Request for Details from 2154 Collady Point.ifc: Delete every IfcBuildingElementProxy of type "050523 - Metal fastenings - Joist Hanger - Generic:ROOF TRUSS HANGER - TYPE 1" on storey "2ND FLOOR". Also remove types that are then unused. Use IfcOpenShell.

First a look at what the model holds.

```python
import ifcopenshell
import ifcopenshell.util.element

model = ifcopenshell.open("Details from 2154 Collady Point.ifc")
print(model.schema)
storey = next(s for s in model.by_type("IfcBuildingStorey") if s.Name == "2ND FLOOR")
proxies = [e for e in ifcopenshell.util.element.get_decomposition(storey) if e.is_a("IfcBuildingElementProxy")]
seen = {}
for e in proxies:
    element_type = ifcopenshell.util.element.get_type(e)
    name = element_type.Name if element_type not in (None, e) else None
    seen[name] = seen.get(name, 0) + 1
for name, count in sorted(seen.items(), key=str):
    print(count, "x", name)
```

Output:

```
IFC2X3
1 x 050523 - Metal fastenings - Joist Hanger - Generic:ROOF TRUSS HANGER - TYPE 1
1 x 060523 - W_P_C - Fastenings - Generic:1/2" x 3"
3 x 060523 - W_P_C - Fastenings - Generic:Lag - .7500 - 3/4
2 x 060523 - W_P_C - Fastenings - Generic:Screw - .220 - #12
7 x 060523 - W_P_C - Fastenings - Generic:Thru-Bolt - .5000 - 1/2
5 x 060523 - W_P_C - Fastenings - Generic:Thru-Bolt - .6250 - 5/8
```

```python
import ifcopenshell
import ifcopenshell.api.root
import ifcopenshell.util.element

model = ifcopenshell.open("Details from 2154 Collady Point.ifc")

storey = next(s for s in model.by_type("IfcBuildingStorey") if s.Name == "2ND FLOOR")
proxies = [e for e in ifcopenshell.util.element.get_decomposition(storey) if e.is_a("IfcBuildingElementProxy")]
targets = [e for e in proxies if (t := ifcopenshell.util.element.get_type(e)) not in (None, e) and t.Name == "050523 - Metal fastenings - Joist Hanger - Generic:ROOF TRUSS HANGER - TYPE 1"]
types = {ifcopenshell.util.element.get_type(e) for e in targets} - {None, *targets}

for e in targets:
    ifcopenshell.api.root.remove_product(model, product=e)
print(len(targets), "removed")

unused = [t for t in types if not ifcopenshell.util.element.get_types(t)]
for t in unused:
    ifcopenshell.api.root.remove_product(model, product=t)
print(len(unused), "unused types removed")

model.write("Details from 2154 Collady Point_edited.ifc")
```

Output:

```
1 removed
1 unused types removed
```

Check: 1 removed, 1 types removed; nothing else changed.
